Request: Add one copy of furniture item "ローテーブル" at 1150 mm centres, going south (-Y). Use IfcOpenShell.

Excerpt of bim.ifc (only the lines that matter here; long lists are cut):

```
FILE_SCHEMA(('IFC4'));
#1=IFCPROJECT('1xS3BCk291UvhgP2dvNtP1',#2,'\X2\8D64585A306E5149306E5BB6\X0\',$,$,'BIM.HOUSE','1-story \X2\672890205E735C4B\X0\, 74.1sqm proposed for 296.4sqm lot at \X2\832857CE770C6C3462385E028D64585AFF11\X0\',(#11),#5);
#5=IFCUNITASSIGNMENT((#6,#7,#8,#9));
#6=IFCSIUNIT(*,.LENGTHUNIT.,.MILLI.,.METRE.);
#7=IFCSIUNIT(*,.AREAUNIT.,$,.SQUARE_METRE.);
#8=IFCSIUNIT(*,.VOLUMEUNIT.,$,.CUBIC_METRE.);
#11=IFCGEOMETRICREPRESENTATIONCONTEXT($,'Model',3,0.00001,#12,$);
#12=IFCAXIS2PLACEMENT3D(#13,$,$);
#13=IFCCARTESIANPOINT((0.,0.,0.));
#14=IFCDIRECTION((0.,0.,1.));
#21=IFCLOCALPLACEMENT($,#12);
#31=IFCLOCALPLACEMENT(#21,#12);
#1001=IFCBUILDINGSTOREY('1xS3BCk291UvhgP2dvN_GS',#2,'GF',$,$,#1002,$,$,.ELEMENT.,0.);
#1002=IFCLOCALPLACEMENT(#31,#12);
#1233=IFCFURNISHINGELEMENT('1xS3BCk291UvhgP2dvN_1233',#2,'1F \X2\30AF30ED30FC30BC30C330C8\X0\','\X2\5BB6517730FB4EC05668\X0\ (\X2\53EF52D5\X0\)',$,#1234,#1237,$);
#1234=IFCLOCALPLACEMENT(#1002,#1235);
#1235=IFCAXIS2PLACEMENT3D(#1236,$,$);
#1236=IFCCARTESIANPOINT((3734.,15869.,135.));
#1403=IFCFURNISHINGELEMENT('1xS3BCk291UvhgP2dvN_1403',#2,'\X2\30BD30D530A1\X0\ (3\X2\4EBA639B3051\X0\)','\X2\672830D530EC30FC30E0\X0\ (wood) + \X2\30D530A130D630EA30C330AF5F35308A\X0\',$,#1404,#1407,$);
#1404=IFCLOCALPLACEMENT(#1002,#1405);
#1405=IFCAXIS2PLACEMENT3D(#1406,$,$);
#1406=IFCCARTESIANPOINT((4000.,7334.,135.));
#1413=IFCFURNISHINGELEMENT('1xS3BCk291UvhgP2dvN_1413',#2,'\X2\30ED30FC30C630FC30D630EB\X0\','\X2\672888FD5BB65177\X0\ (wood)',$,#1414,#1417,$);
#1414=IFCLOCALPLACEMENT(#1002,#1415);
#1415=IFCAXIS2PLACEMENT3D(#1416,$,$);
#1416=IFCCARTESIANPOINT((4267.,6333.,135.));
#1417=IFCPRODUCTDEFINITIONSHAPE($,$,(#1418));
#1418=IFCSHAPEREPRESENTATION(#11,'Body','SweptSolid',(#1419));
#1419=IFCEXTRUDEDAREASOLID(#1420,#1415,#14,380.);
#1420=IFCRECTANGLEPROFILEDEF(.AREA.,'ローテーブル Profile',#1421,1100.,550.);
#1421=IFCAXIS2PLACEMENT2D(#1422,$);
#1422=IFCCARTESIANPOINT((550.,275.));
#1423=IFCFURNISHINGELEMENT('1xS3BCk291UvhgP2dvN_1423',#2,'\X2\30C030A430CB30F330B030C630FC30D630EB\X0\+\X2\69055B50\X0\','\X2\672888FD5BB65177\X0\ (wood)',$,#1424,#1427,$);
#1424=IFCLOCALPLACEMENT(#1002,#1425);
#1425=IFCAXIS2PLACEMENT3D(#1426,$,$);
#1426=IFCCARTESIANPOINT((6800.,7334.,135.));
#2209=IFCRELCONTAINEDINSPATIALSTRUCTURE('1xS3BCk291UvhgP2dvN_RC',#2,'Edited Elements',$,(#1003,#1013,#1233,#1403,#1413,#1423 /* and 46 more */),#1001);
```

```python
import numpy as np
import ifcopenshell
import ifcopenshell.api.geometry
import ifcopenshell.api.root
import ifcopenshell.util.element
import ifcopenshell.util.placement
import ifcopenshell.util.unit

model = ifcopenshell.open("bim.ifc")
unit_scale = ifcopenshell.util.unit.calculate_unit_scale(model)


def reuse_history(source, copy):
    """copy_class also copies each property set's owner history, people and application; keep the originals."""
    for rel in copy.IsDefinedBy:
        if rel.is_a("IfcRelDefinesByProperties") and (history := rel.RelatingPropertyDefinition.OwnerHistory):
            rel.RelatingPropertyDefinition.OwnerHistory = source.OwnerHistory
            ifcopenshell.util.element.remove_deep2(model, history)


source = model.by_guid("1xS3BCk291UvhgP2dvN_1413")
base = ifcopenshell.util.placement.get_local_placement(source.ObjectPlacement)
step = np.array([0.0, -1.0, 0.0]) * 1.15 / unit_scale

for i in range(1, 2):
    copy = ifcopenshell.api.root.copy_class(model, product=source)
    copy.Representation = ifcopenshell.util.element.copy_deep(
        model, source.Representation, exclude=["IfcGeometricRepresentationContext", "IfcRepresentationMap"]
    )
    reuse_history(source, copy)
    matrix = base.copy()
    matrix[:3, 3] += i * step
    print("added at", matrix[:3, 3].round(3) + 0.0)
    ifcopenshell.api.geometry.edit_object_placement(model, product=copy, matrix=matrix, is_si=False)

model.write("bim_edited.ifc")
```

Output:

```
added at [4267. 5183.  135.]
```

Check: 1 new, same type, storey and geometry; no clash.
